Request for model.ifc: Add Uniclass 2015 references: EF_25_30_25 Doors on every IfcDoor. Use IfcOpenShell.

First a look at what the model holds.

```python
import ifcopenshell

model = ifcopenshell.open("model.ifc")
print(model.schema)
print("classifications:", [c.Name for c in model.by_type("IfcClassification")])
for ifc_class in ("IfcDoor", "IfcRoof", "IfcStair", "IfcWall", "IfcWindow"):
    print(ifc_class, len(model.by_type(ifc_class)))
```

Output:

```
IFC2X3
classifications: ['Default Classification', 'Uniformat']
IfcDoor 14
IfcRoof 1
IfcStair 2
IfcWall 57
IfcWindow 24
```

```python
import ifcopenshell
import ifcopenshell.api.classification

model = ifcopenshell.open("model.ifc")

# IFC2X3 requires Source and Edition and has no link from the project to the system.
system = model.create_entity("IfcClassification", Source="NBS", Edition="2015", Name="Uniclass 2015")

codes = {
    "IfcDoor": ("EF_25_30_25", "Doors"),
}
for ifc_class, (code, name) in codes.items():
    products = model.by_type(ifc_class)
    ifcopenshell.api.classification.add_reference(
        model, products=products, classification=system, identification=code, name=name
    )
    print(code, len(products))

model.write("model_updated.ifc")
```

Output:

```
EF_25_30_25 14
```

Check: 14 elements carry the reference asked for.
